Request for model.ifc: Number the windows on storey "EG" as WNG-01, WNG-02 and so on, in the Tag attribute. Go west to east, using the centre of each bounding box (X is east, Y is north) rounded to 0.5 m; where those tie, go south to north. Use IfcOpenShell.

First a look at what the model holds.

```python
import ifcopenshell
import ifcopenshell.util.element
import ifcopenshell.util.placement

model = ifcopenshell.open("model.ifc")
print(model.schema)
storey = next(s for s in model.by_type("IfcBuildingStorey") if s.Name == "EG")
windows = [e for e in ifcopenshell.util.element.get_decomposition(storey) if e.is_a("IfcWindow")]
for e in sorted(windows, key=lambda e: e.id()):
    origin = ifcopenshell.util.placement.get_local_placement(e.ObjectPlacement)[:3, 3]
    print(e.id(), e.Tag, e.Name, origin.round(2) + 0.0, sep=" | ")
```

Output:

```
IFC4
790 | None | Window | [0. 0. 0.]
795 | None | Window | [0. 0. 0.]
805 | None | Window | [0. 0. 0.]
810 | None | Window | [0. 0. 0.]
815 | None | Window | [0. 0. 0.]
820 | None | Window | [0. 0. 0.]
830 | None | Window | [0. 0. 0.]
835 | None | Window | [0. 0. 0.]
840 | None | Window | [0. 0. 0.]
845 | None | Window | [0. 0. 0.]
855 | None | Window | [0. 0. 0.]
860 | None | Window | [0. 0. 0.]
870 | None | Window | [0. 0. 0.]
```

```python
import ifcopenshell
import ifcopenshell.geom
import ifcopenshell.util.element
import ifcopenshell.util.shape

model = ifcopenshell.open("model.ifc")
settings = ifcopenshell.geom.settings()
settings.set("use-world-coords", True)


def centre(element):
    shape = ifcopenshell.geom.create_shape(settings, element)
    return ifcopenshell.util.shape.get_bbox_centroid(shape.geometry)


storey = next(s for s in model.by_type("IfcBuildingStorey") if s.Name == "EG")
windows = [e for e in ifcopenshell.util.element.get_decomposition(storey) if e.is_a("IfcWindow")]

# Insertion points can sit at a corner or the storey origin, so sort by the geometry (in metres).
centres = {e: centre(e) for e in windows}
windows.sort(key=lambda e: (round(centres[e][0] / 0.5), centres[e][1]))

for i, e in enumerate(windows, start=1):
    number = f"WNG-{i:02d}"
    e.Tag = number
    print(e.id(), number)

model.write("model_updated.ifc")
```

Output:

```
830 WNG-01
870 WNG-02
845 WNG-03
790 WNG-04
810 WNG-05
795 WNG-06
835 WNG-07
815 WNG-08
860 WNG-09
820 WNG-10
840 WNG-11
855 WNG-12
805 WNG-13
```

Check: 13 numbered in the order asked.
